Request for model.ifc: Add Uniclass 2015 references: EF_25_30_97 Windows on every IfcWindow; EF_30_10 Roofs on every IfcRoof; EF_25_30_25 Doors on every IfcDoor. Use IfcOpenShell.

First a look at what the model holds.

```python
import ifcopenshell

model = ifcopenshell.open("model.ifc")
print(model.schema)
print("classifications:", [c.Name for c in model.by_type("IfcClassification")])
for ifc_class in ("IfcDoor", "IfcRoof", "IfcStair", "IfcWall", "IfcWindow"):
    print(ifc_class, len(model.by_type(ifc_class)))
```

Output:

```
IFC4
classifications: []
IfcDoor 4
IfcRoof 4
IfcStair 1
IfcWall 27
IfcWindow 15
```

```python
import ifcopenshell
import ifcopenshell.api.classification

model = ifcopenshell.open("model.ifc")

system = ifcopenshell.api.classification.add_classification(model, classification="Uniclass 2015")

codes = {
    "IfcWindow": ("EF_25_30_97", "Windows"),
    "IfcRoof": ("EF_30_10", "Roofs"),
    "IfcDoor": ("EF_25_30_25", "Doors"),
}
for ifc_class, (code, name) in codes.items():
    products = model.by_type(ifc_class)
    ifcopenshell.api.classification.add_reference(
        model, products=products, classification=system, identification=code, name=name
    )
    print(code, len(products))

model.write("model_edited.ifc")
```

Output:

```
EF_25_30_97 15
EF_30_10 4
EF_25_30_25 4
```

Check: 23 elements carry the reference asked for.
